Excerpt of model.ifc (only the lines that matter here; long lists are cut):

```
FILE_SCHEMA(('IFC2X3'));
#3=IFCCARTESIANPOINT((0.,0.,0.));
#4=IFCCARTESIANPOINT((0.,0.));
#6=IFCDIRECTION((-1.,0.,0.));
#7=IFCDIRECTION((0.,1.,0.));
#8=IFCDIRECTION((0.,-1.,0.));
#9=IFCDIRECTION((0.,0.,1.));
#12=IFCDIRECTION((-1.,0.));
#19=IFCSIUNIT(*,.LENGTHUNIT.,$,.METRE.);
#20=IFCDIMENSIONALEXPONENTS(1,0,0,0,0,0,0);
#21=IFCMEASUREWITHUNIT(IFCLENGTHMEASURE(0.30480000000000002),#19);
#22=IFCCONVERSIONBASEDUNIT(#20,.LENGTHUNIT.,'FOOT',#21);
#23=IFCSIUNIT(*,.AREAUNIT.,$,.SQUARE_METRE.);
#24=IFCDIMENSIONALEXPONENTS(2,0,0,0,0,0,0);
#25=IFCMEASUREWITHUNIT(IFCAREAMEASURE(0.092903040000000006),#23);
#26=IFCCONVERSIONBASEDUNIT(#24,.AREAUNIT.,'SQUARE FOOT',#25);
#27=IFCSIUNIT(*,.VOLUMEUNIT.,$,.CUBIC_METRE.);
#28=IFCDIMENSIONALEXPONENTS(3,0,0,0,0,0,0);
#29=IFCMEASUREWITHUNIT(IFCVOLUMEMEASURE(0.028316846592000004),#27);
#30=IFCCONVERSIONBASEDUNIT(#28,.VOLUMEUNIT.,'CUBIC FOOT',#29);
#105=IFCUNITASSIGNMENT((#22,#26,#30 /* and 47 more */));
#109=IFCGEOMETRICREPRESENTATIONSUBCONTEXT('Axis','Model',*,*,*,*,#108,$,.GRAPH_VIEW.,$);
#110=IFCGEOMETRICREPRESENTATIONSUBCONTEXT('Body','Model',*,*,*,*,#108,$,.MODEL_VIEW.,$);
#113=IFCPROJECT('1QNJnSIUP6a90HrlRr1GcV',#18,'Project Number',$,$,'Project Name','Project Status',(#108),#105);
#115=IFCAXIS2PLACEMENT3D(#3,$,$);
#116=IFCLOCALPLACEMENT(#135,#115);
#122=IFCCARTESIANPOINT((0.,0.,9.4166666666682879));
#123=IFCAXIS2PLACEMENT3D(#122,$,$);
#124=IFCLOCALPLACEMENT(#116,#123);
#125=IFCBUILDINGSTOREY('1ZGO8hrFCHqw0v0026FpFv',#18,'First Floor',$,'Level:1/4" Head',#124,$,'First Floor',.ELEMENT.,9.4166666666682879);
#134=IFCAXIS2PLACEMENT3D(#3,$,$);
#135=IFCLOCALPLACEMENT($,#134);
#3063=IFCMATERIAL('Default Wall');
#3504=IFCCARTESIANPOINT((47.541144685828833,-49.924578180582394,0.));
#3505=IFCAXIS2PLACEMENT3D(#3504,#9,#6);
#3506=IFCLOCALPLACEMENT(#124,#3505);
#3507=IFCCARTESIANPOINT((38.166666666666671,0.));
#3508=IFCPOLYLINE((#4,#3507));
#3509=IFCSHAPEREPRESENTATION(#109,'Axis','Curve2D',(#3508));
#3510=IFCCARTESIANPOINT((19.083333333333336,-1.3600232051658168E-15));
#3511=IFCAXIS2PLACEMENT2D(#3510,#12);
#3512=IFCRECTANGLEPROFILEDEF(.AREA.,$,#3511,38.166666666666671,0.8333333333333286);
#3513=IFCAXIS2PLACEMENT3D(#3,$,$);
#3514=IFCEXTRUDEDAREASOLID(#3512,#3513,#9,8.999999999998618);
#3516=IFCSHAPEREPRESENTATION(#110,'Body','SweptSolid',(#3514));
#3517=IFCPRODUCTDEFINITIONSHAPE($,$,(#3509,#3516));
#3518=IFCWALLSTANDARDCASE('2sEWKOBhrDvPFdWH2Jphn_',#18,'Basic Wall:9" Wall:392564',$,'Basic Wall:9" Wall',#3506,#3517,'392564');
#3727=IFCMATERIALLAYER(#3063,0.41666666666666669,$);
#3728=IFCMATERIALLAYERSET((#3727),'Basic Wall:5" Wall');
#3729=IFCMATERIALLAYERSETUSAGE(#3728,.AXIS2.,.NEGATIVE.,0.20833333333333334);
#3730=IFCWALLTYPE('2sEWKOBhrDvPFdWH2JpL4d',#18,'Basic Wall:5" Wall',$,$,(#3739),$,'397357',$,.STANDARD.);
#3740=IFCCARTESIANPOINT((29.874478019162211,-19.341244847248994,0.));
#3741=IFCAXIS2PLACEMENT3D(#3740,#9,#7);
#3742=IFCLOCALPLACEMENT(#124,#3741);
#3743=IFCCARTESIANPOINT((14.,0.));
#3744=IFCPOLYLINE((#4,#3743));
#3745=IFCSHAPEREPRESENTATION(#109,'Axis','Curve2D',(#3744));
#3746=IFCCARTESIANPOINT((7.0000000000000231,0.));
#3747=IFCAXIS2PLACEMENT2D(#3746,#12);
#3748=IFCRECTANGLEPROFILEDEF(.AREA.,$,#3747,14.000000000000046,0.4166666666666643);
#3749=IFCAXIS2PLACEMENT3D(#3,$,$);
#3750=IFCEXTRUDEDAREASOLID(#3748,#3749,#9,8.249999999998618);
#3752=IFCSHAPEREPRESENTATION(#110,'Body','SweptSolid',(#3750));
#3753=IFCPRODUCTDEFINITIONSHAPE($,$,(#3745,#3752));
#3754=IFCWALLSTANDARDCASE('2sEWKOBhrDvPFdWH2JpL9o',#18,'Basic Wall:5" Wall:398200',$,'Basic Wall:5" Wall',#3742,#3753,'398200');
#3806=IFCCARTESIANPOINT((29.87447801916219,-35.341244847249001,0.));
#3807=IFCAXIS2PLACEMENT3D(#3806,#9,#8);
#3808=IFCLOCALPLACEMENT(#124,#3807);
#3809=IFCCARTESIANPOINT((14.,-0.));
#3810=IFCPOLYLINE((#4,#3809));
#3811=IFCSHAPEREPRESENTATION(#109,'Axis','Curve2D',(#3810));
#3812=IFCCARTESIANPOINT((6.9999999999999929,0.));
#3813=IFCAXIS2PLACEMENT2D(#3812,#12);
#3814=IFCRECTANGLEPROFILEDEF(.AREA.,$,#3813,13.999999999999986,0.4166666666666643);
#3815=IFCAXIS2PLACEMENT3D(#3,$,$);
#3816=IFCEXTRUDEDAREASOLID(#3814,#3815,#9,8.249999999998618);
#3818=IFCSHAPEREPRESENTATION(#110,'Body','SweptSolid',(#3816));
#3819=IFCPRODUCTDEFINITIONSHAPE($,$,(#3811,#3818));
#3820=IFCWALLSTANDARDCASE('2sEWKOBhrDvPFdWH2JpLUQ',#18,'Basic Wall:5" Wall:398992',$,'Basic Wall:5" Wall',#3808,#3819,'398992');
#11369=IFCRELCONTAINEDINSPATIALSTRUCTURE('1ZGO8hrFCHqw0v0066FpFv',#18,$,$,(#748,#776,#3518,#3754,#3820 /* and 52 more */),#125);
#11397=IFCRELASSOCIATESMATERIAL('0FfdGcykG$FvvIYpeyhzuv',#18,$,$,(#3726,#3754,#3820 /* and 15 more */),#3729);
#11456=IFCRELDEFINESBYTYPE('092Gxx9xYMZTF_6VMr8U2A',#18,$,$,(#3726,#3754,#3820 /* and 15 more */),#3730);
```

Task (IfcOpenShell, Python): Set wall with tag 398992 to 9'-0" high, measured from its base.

```python
import ifcopenshell
import ifcopenshell.geom
import ifcopenshell.util.representation
import ifcopenshell.util.shape
import ifcopenshell.util.unit

model = ifcopenshell.open("model.ifc")
unit_scale = ifcopenshell.util.unit.calculate_unit_scale(model)
settings = ifcopenshell.geom.settings()


def volume(element):
    """Net volume in cubic metres, openings subtracted."""
    shape = ifcopenshell.geom.create_shape(settings, element)
    return ifcopenshell.util.shape.get_volume(shape.geometry)


wall = model.by_id(3820)
before = volume(wall)

body = ifcopenshell.util.representation.get_representation(wall, "Model", "Body")
solid = body.Items[0]
old_height = solid.Depth
solid.Depth = 108 * 0.0254 / unit_scale
after = volume(wall)

print(f"height {old_height:g} -> {solid.Depth:g}, volume {before:.3f} -> {after:.3f} m3")

model.write("model_v2.ifc")
```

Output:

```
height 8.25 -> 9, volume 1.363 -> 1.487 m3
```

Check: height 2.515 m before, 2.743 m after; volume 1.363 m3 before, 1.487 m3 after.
